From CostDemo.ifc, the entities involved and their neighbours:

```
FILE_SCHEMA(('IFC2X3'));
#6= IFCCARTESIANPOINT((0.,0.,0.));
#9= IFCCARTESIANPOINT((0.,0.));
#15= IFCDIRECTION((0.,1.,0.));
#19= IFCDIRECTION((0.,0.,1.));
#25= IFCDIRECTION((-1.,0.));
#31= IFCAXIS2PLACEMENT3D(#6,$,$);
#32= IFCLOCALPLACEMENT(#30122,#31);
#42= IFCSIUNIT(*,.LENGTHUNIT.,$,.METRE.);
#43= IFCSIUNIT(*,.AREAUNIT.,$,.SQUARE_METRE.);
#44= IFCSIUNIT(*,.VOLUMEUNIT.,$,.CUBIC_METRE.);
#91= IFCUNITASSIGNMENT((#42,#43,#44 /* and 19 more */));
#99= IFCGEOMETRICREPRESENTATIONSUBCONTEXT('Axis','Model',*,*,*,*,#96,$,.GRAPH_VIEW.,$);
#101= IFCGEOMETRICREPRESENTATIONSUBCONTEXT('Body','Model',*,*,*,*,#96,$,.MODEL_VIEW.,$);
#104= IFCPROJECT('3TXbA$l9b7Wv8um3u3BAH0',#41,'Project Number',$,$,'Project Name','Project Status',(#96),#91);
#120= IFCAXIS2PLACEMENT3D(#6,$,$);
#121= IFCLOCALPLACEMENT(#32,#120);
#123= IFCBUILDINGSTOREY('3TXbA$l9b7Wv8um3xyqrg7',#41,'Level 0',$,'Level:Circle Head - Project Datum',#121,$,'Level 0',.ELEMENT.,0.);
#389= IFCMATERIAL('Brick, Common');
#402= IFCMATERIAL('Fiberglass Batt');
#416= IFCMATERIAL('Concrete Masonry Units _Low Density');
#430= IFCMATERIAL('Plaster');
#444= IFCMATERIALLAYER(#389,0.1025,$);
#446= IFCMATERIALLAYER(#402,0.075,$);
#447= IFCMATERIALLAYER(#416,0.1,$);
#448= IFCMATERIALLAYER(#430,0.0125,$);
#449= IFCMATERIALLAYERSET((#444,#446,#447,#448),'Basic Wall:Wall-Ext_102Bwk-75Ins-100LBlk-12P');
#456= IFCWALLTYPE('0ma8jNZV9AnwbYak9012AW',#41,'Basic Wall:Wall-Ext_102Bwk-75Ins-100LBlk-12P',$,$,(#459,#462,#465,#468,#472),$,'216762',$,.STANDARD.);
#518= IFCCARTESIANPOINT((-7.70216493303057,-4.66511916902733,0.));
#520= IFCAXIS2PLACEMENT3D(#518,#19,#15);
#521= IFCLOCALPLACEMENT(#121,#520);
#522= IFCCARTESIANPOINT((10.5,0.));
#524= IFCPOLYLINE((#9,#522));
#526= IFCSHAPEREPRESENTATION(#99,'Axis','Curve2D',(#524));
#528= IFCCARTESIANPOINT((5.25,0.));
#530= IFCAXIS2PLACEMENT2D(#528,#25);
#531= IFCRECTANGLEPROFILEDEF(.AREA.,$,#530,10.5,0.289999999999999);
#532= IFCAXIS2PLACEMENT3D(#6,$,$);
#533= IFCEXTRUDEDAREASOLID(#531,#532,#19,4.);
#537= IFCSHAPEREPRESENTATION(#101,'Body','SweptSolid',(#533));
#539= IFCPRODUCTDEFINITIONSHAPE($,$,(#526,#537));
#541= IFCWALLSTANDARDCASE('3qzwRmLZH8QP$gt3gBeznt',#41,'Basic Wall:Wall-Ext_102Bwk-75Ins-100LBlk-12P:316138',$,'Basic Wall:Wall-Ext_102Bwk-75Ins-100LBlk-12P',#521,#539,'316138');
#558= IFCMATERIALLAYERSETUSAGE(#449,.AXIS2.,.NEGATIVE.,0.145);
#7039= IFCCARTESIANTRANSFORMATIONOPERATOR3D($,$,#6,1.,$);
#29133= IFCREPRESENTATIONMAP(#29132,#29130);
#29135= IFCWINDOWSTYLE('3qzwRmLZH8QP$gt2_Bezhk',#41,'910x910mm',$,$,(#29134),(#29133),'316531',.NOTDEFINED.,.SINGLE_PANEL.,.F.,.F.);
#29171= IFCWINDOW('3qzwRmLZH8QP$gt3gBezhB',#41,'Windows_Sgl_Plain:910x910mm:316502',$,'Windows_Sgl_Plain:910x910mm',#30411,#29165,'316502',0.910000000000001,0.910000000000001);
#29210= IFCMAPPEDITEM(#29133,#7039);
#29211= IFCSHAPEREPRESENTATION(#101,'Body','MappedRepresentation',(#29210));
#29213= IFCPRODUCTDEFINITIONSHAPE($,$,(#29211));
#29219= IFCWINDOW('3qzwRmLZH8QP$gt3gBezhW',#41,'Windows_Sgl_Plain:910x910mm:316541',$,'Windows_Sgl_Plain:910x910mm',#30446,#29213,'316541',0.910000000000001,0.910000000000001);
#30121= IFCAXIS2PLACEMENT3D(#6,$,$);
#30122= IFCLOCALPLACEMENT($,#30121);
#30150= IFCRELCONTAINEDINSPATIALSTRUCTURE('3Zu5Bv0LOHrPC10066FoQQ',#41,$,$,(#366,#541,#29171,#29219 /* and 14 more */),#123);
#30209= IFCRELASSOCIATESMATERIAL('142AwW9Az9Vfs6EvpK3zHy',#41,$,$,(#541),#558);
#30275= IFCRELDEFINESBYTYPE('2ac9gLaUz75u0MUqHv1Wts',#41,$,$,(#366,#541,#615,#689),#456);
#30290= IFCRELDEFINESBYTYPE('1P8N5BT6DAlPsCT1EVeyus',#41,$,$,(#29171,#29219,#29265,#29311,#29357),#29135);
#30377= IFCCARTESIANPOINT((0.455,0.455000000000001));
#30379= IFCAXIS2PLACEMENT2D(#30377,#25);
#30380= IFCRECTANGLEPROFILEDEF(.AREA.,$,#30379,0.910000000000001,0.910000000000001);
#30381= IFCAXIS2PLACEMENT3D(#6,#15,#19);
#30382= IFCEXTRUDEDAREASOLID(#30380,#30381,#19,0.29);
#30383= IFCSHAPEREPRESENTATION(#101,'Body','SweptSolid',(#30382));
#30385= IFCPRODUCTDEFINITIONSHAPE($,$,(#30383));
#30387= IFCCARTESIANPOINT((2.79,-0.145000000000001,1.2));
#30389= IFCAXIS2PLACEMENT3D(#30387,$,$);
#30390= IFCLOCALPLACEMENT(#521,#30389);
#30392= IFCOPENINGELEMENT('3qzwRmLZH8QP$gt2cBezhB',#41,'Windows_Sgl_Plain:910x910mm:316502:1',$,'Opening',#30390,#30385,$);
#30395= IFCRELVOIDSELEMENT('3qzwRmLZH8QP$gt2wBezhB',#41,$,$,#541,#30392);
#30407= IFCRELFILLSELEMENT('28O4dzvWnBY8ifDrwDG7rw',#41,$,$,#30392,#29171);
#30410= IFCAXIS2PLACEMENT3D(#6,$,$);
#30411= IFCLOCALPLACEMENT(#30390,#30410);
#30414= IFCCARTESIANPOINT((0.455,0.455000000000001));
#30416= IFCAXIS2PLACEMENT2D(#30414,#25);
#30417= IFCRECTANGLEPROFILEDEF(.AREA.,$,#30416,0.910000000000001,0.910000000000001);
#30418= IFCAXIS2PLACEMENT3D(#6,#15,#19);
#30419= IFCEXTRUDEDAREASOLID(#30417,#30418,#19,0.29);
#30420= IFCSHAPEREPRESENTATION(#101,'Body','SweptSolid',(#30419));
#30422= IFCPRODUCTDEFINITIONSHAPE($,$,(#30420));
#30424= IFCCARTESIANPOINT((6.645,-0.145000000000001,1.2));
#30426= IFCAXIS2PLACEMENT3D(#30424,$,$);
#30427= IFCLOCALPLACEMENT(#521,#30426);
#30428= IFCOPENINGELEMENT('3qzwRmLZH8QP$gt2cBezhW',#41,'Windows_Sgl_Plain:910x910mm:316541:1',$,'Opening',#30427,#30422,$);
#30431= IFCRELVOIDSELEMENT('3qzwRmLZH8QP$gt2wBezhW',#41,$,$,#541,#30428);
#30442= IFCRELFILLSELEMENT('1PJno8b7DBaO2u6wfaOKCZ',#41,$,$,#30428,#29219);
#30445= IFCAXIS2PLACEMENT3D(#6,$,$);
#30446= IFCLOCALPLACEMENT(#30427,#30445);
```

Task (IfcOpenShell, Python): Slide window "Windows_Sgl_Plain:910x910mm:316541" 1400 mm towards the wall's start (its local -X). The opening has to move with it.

```python
import ifcopenshell
import ifcopenshell.api.geometry
import ifcopenshell.util.placement

model = ifcopenshell.open("CostDemo.ifc")

window = model.by_guid("3qzwRmLZH8QP$gt3gBezhW")
opening = window.FillsVoids[0].RelatingOpeningElement
wall = opening.VoidsElements[0].RelatingBuildingElement

wall_matrix = ifcopenshell.util.placement.get_local_placement(wall.ObjectPlacement)
shift = wall_matrix[:3, 0] * -1.4
before = ifcopenshell.util.placement.get_local_placement(window.ObjectPlacement)[:3, 3].copy()

# The window is placed relative to its opening, so it follows when the opening moves.
matrix = ifcopenshell.util.placement.get_local_placement(opening.ObjectPlacement)
matrix[:3, 3] += shift
ifcopenshell.api.geometry.edit_object_placement(
    model, product=opening, matrix=matrix, is_si=False, should_transform_children=True
)

after = ifcopenshell.util.placement.get_local_placement(window.ObjectPlacement)[:3, 3]
print("window moved by", (after - before).round(3) + 0.0)

model.write("CostDemo_v2.ifc")
```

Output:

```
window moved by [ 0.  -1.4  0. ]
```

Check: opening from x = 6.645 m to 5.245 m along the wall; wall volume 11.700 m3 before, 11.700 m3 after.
